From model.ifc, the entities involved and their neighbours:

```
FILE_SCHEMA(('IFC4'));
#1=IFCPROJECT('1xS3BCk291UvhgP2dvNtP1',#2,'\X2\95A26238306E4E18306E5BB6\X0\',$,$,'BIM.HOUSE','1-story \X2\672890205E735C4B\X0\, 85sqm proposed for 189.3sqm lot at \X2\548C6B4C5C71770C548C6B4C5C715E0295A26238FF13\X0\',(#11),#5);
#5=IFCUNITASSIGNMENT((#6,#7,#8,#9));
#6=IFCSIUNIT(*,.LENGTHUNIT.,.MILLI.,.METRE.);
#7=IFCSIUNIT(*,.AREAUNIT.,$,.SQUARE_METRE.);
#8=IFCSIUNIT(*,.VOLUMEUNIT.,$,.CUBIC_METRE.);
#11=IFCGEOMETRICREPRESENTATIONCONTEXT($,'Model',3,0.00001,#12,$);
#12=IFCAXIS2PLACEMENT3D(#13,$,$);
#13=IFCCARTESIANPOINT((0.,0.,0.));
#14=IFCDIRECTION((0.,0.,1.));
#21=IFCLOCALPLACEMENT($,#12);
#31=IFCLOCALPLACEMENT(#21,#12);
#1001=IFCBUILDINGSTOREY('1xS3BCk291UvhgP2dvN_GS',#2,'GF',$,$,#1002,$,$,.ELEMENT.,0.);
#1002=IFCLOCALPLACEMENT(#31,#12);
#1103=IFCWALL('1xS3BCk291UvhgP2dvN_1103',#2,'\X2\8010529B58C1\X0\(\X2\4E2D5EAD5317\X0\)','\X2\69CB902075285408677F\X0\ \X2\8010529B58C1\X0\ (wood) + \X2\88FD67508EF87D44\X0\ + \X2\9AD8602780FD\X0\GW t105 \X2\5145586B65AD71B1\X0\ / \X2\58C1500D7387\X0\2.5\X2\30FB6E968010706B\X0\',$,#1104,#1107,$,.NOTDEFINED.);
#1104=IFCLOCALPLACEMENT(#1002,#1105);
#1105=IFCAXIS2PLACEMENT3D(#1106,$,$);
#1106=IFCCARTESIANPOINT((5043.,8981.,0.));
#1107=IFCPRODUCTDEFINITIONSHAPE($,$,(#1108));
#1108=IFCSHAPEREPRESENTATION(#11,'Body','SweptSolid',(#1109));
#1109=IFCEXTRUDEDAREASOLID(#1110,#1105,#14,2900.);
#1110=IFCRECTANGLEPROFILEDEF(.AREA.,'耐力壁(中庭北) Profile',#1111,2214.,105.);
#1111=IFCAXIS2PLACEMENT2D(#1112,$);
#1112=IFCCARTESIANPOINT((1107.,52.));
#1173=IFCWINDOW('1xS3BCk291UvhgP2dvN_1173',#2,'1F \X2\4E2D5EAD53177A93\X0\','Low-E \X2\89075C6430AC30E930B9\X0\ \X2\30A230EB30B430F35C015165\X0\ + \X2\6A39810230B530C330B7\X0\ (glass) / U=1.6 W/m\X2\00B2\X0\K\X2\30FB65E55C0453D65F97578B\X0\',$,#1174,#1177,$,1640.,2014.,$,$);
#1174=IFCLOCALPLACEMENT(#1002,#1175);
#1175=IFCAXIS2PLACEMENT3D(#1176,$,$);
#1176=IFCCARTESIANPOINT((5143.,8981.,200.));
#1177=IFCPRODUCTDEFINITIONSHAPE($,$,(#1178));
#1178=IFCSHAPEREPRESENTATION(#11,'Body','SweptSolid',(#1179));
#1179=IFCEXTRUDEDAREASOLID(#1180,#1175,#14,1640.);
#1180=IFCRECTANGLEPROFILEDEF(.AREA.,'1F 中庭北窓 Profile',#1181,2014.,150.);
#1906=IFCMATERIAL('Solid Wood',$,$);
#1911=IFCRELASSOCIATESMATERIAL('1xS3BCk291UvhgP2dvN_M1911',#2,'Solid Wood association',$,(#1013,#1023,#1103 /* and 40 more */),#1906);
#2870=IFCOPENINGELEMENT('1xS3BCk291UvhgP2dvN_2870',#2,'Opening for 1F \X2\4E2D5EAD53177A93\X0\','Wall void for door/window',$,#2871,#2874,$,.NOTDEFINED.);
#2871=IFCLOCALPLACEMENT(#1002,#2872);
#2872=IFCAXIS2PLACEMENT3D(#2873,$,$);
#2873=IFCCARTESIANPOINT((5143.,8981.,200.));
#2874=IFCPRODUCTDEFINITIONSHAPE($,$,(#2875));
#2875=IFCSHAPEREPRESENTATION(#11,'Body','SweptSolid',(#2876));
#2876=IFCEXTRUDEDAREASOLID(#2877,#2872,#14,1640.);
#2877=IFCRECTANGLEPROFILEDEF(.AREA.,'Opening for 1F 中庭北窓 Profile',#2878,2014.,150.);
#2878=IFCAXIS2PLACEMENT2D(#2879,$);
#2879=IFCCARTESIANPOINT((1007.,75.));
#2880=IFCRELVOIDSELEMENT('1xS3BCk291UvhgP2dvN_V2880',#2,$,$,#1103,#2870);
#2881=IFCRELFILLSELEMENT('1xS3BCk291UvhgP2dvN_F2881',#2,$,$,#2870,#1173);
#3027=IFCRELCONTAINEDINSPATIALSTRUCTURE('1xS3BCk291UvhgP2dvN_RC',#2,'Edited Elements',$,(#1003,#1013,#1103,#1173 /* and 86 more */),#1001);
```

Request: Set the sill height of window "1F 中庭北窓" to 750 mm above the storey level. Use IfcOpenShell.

```python
import numpy as np
import ifcopenshell
import ifcopenshell.api.geometry
import ifcopenshell.geom
import ifcopenshell.util.element
import ifcopenshell.util.placement
import ifcopenshell.util.shape
import ifcopenshell.util.unit

model = ifcopenshell.open("model.ifc")
unit_scale = ifcopenshell.util.unit.calculate_unit_scale(model)

window = model.by_guid("1xS3BCk291UvhgP2dvN_1173")
opening = window.FillsVoids[0].RelatingOpeningElement
storey = ifcopenshell.util.element.get_container(window, ifc_class="IfcBuildingStorey")
level = ifcopenshell.util.placement.get_local_placement(storey.ObjectPlacement)[2, 3]

# The opening's origin need not be at the sill, so measure its lowest point.
shape = ifcopenshell.geom.create_shape(ifcopenshell.geom.settings(), opening)
bottom = ifcopenshell.util.shape.get_shape_bottom_elevation(shape, shape.geometry) / unit_scale
dz = level + 0.75 / unit_scale - bottom

shift = np.array([0.0, 0.0, dz])
# The window is not placed relative to its opening, so move both.
for product in (opening, window):
    matrix = ifcopenshell.util.placement.get_local_placement(product.ObjectPlacement)
    matrix[:3, 3] += shift
    ifcopenshell.api.geometry.edit_object_placement(model, product=product, matrix=matrix, is_si=False)

print(f"moved by {dz * unit_scale:+.3f} m")

model.write("model_v2.ifc")
```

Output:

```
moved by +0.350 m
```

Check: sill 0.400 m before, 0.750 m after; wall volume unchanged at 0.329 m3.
